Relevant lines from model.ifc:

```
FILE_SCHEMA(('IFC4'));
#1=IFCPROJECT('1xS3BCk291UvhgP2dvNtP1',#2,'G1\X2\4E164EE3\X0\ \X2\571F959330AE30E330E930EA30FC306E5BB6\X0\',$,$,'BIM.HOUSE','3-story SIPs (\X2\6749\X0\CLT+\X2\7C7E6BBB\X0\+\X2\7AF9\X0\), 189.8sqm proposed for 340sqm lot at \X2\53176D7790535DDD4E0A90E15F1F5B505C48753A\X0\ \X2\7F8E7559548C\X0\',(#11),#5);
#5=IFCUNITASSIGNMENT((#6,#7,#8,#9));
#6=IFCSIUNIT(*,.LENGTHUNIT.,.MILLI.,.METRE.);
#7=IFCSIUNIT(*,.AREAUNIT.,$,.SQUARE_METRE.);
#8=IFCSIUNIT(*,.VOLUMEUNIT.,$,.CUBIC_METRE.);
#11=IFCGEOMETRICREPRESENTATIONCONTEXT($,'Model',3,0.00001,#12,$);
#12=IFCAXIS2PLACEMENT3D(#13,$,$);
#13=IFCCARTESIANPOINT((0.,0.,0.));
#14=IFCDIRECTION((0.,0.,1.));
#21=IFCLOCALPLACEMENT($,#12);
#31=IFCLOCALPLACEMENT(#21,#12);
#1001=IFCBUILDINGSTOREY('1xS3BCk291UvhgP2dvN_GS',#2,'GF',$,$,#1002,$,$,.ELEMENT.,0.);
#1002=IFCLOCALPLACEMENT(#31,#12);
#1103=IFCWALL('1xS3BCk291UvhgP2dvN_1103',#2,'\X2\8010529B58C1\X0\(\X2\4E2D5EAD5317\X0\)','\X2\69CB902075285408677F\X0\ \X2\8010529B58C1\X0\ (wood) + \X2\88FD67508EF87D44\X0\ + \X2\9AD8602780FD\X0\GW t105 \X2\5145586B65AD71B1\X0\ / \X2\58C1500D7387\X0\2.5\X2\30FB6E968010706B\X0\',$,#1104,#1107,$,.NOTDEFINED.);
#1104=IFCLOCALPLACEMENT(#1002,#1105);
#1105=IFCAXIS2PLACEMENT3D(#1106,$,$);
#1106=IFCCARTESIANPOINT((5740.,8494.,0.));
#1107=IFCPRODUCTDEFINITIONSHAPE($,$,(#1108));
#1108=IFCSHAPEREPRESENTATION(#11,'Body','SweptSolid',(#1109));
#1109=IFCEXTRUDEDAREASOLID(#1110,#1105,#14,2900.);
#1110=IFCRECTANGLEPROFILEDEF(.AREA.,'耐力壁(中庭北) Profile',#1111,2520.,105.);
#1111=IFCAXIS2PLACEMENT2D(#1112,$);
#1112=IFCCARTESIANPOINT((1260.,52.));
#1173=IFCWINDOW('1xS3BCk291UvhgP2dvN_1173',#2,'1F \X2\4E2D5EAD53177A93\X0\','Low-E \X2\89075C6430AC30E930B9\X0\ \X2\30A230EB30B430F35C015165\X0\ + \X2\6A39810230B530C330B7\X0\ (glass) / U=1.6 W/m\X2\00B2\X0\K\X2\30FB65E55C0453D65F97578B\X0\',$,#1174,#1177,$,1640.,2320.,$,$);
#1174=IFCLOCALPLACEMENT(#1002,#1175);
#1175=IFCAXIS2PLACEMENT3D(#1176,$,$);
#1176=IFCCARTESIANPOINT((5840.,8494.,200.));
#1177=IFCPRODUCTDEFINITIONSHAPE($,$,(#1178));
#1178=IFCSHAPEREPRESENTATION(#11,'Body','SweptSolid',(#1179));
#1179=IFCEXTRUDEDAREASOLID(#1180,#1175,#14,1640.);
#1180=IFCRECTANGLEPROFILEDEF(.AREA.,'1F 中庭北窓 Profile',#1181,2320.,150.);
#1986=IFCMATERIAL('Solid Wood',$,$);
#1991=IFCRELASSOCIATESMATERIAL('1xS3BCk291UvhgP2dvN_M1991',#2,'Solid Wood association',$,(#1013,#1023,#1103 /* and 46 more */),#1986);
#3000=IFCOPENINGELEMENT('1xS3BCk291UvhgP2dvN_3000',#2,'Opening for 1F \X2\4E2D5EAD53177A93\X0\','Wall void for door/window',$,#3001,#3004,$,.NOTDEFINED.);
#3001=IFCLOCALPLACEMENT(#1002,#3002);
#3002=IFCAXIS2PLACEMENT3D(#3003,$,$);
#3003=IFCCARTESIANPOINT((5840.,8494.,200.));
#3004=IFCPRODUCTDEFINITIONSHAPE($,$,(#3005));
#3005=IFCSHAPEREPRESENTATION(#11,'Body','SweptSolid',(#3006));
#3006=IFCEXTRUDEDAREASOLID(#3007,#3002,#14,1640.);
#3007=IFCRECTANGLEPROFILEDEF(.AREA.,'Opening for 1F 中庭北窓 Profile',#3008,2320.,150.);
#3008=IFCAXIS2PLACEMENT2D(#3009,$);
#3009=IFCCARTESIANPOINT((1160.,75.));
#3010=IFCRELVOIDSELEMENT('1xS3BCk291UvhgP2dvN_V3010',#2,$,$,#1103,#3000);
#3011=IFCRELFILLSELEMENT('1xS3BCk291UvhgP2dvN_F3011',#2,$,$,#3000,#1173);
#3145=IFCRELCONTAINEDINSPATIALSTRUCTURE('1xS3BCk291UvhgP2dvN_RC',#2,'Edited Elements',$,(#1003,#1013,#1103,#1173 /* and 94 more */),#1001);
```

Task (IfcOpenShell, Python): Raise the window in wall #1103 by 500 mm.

```python
import numpy as np
import ifcopenshell
import ifcopenshell.api.geometry
import ifcopenshell.util.placement
import ifcopenshell.util.unit

model = ifcopenshell.open("model.ifc")
unit_scale = ifcopenshell.util.unit.calculate_unit_scale(model)

window = model.by_guid("1xS3BCk291UvhgP2dvN_1173")
opening = window.FillsVoids[0].RelatingOpeningElement
dz = 0.5 / unit_scale

shift = np.array([0.0, 0.0, dz])
# The window is not placed relative to its opening, so move both.
for product in (opening, window):
    matrix = ifcopenshell.util.placement.get_local_placement(product.ObjectPlacement)
    matrix[:3, 3] += shift
    ifcopenshell.api.geometry.edit_object_placement(model, product=product, matrix=matrix, is_si=False)

print(f"moved by {dz * unit_scale:+.3f} m")

model.write("model_rev.ifc")
```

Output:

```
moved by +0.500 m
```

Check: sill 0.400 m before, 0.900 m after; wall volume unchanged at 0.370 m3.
